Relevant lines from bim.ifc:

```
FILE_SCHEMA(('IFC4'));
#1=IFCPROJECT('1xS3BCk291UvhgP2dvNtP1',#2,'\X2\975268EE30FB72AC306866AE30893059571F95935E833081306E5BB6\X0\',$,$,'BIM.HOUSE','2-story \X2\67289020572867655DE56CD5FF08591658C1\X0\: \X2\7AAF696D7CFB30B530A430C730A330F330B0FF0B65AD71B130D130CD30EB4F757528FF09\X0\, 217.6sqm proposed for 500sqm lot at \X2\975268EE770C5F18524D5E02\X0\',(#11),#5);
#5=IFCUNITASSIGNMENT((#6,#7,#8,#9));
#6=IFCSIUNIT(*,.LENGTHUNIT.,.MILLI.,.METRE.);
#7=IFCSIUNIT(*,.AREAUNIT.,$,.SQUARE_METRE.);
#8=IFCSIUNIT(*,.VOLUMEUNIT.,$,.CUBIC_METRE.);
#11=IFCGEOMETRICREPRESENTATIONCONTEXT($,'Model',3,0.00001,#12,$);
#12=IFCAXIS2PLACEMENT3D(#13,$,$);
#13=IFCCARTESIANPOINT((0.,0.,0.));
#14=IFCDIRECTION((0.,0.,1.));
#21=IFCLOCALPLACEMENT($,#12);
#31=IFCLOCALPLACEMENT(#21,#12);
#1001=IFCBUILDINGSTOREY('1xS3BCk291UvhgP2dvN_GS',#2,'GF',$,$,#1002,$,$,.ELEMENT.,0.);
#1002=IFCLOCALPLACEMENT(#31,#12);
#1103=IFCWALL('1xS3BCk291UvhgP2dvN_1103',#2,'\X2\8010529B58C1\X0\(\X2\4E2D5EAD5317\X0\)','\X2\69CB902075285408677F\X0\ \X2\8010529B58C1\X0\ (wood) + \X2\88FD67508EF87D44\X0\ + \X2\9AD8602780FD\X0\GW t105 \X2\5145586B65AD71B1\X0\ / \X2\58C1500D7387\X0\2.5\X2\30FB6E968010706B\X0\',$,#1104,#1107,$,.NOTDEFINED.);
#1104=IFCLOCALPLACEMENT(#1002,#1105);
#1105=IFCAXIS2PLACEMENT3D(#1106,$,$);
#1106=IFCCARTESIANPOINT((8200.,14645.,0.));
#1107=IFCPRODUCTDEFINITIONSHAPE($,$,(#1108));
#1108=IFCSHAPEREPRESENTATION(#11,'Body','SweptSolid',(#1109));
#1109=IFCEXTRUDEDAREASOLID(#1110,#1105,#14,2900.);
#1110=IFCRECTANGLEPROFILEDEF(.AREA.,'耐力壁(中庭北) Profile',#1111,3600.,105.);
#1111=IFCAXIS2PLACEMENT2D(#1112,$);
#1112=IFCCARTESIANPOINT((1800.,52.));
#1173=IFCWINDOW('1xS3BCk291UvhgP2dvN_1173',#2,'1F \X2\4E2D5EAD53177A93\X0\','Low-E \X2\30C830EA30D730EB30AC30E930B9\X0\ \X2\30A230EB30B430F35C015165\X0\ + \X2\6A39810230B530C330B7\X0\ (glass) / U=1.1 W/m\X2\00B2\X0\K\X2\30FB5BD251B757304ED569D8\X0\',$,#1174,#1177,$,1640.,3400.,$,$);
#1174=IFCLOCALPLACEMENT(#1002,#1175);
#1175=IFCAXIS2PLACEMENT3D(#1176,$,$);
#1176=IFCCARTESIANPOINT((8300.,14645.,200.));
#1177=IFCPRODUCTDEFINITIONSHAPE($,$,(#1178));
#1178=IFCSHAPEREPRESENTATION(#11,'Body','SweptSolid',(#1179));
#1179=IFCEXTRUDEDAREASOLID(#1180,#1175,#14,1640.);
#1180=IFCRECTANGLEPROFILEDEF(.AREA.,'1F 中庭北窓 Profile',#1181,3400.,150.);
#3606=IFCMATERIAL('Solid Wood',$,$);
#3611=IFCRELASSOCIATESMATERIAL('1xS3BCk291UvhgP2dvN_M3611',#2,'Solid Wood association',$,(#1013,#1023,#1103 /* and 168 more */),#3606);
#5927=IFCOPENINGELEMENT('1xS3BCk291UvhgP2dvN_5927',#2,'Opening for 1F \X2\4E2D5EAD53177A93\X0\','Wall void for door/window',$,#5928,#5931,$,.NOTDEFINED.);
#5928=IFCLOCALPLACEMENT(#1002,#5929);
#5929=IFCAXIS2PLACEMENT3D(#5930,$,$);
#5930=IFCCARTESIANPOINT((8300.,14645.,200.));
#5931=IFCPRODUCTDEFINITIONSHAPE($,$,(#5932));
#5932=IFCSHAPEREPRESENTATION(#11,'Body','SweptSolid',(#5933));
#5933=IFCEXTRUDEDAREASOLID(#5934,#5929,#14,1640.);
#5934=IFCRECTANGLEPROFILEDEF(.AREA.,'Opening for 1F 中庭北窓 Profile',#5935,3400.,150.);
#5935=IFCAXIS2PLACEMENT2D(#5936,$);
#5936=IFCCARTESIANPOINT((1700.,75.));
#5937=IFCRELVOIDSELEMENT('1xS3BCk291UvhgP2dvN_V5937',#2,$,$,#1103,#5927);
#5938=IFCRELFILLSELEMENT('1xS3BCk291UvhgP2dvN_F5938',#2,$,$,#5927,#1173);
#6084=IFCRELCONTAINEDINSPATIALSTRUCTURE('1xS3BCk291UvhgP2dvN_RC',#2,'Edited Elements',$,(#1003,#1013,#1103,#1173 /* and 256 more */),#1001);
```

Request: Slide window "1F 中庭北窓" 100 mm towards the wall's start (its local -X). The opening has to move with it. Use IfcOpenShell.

```python
import ifcopenshell
import ifcopenshell.api.geometry
import ifcopenshell.util.placement

model = ifcopenshell.open("bim.ifc")

window = model.by_guid("1xS3BCk291UvhgP2dvN_1173")
opening = window.FillsVoids[0].RelatingOpeningElement
wall = opening.VoidsElements[0].RelatingBuildingElement

wall_matrix = ifcopenshell.util.placement.get_local_placement(wall.ObjectPlacement)
shift = wall_matrix[:3, 0] * -100.0
before = ifcopenshell.util.placement.get_local_placement(window.ObjectPlacement)[:3, 3].copy()

# The window is not placed relative to its opening, so move both.
for product in (opening, window):
    matrix = ifcopenshell.util.placement.get_local_placement(product.ObjectPlacement)
    matrix[:3, 3] += shift
    ifcopenshell.api.geometry.edit_object_placement(model, product=product, matrix=matrix, is_si=False)

after = ifcopenshell.util.placement.get_local_placement(window.ObjectPlacement)[:3, 3]
print("window moved by", (after - before).round(3) + 0.0)

model.write("bim_v2.ifc")
```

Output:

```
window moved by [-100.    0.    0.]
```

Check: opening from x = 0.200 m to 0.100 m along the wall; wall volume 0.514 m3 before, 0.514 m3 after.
